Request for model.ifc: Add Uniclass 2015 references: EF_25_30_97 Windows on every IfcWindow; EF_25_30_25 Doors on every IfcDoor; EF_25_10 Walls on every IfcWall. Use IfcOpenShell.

First a look at what the model holds.

```python
import ifcopenshell

model = ifcopenshell.open("model.ifc")
print(model.schema)
print("classifications:", [c.Name for c in model.by_type("IfcClassification")])
for ifc_class in ("IfcDoor", "IfcRoof", "IfcStair", "IfcWall", "IfcWindow"):
    print(ifc_class, len(model.by_type(ifc_class)))
```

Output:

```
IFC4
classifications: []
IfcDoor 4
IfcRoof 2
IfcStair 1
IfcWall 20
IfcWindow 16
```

```python
import ifcopenshell
import ifcopenshell.api.classification

model = ifcopenshell.open("model.ifc")

system = ifcopenshell.api.classification.add_classification(model, classification="Uniclass 2015")

codes = {
    "IfcWindow": ("EF_25_30_97", "Windows"),
    "IfcDoor": ("EF_25_30_25", "Doors"),
    "IfcWall": ("EF_25_10", "Walls"),
}
for ifc_class, (code, name) in codes.items():
    products = model.by_type(ifc_class)
    ifcopenshell.api.classification.add_reference(
        model, products=products, classification=system, identification=code, name=name
    )
    print(code, len(products))

model.write("model_edited.ifc")
```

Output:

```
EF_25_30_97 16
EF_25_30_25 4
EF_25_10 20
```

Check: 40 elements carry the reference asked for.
